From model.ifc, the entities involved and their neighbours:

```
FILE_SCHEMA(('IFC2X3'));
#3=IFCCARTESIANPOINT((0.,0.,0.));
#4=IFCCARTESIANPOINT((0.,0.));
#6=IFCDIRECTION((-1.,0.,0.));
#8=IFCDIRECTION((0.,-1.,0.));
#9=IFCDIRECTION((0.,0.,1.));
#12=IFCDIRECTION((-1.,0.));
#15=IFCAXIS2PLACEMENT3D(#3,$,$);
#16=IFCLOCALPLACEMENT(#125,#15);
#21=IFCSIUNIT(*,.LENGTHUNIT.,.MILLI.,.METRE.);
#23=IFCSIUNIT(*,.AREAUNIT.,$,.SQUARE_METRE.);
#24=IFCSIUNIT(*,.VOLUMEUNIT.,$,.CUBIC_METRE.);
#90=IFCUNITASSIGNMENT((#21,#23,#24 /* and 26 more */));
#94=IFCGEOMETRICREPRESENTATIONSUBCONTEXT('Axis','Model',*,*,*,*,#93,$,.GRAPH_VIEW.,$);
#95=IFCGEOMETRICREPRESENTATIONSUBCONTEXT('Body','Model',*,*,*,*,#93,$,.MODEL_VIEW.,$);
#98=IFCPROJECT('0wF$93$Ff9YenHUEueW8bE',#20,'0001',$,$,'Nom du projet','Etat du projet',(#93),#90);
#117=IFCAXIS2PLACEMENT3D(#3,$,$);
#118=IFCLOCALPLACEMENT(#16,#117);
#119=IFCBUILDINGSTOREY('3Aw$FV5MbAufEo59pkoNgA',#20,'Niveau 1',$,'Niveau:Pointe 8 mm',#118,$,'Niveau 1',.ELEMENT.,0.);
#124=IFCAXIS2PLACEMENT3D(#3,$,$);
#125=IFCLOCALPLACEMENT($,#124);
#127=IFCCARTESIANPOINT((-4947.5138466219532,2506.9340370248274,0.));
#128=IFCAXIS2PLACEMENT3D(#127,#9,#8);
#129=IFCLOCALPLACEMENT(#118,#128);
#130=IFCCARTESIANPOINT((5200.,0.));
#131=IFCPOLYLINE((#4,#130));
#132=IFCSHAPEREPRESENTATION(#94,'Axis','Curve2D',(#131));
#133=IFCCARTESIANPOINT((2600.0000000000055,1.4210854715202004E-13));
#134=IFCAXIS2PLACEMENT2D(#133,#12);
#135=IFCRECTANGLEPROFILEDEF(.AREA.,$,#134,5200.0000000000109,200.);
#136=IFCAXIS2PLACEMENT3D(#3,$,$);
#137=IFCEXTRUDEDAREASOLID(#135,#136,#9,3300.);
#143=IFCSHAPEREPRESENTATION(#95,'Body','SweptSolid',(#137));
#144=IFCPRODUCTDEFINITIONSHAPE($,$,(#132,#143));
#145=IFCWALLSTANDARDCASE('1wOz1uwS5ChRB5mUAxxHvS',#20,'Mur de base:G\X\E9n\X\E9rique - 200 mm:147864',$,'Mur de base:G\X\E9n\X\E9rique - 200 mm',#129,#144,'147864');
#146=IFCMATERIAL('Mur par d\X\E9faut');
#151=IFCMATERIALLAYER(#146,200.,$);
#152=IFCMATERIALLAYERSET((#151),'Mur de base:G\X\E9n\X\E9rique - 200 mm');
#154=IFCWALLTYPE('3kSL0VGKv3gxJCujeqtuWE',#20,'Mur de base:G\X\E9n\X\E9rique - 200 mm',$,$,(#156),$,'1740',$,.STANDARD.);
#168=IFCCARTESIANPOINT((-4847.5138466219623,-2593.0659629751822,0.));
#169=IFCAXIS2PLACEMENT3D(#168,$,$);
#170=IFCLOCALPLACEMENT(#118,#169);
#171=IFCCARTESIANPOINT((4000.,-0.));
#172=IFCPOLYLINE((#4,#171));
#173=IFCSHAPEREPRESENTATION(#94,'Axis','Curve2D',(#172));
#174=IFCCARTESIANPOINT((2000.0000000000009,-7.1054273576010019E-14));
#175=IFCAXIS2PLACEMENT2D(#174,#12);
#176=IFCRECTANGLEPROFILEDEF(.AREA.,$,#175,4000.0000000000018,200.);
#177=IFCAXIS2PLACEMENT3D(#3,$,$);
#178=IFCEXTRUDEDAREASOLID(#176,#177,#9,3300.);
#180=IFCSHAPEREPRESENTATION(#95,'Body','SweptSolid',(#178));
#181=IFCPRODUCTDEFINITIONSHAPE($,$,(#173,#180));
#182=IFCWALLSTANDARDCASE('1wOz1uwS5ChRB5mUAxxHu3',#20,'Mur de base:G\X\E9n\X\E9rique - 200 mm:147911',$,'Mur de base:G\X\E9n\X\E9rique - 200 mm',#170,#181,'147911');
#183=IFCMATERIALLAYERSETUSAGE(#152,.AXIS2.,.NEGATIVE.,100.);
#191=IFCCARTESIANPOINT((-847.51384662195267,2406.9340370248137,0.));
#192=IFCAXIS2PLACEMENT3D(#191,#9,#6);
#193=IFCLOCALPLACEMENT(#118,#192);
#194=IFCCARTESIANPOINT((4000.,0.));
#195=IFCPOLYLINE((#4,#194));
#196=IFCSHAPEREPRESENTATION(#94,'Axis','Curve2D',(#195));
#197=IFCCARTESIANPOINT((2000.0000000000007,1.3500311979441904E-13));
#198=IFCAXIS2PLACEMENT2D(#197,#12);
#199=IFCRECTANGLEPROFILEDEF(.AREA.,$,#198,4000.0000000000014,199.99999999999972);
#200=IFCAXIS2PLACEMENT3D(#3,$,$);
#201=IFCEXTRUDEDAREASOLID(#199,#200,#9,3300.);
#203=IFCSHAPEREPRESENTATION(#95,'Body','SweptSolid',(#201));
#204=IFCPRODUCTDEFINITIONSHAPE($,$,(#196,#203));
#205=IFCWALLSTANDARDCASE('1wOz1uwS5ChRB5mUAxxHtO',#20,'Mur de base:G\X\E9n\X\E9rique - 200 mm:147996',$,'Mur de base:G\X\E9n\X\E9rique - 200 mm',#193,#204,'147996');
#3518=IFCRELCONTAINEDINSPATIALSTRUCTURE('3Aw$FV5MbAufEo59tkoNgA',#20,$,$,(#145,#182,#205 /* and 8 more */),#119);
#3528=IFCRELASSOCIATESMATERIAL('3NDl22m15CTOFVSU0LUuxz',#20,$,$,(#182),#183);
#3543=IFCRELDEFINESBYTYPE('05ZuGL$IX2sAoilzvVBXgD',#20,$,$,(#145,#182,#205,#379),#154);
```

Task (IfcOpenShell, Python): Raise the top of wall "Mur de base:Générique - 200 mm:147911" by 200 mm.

```python
import ifcopenshell
import ifcopenshell.geom
import ifcopenshell.util.representation
import ifcopenshell.util.shape

model = ifcopenshell.open("model.ifc")
settings = ifcopenshell.geom.settings()


def volume(element):
    """Net volume in cubic metres, openings subtracted."""
    shape = ifcopenshell.geom.create_shape(settings, element)
    return ifcopenshell.util.shape.get_volume(shape.geometry)


wall = model.by_id(182)
before = volume(wall)

body = ifcopenshell.util.representation.get_representation(wall, "Model", "Body")
solid = body.Items[0]
old_height = solid.Depth
solid.Depth += 200.0
after = volume(wall)

print(f"height {old_height:g} -> {solid.Depth:g}, volume {before:.3f} -> {after:.3f} m3")

model.write("model_updated.ifc")
```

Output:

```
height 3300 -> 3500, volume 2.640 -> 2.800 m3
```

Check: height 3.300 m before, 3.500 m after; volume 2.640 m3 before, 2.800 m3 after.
